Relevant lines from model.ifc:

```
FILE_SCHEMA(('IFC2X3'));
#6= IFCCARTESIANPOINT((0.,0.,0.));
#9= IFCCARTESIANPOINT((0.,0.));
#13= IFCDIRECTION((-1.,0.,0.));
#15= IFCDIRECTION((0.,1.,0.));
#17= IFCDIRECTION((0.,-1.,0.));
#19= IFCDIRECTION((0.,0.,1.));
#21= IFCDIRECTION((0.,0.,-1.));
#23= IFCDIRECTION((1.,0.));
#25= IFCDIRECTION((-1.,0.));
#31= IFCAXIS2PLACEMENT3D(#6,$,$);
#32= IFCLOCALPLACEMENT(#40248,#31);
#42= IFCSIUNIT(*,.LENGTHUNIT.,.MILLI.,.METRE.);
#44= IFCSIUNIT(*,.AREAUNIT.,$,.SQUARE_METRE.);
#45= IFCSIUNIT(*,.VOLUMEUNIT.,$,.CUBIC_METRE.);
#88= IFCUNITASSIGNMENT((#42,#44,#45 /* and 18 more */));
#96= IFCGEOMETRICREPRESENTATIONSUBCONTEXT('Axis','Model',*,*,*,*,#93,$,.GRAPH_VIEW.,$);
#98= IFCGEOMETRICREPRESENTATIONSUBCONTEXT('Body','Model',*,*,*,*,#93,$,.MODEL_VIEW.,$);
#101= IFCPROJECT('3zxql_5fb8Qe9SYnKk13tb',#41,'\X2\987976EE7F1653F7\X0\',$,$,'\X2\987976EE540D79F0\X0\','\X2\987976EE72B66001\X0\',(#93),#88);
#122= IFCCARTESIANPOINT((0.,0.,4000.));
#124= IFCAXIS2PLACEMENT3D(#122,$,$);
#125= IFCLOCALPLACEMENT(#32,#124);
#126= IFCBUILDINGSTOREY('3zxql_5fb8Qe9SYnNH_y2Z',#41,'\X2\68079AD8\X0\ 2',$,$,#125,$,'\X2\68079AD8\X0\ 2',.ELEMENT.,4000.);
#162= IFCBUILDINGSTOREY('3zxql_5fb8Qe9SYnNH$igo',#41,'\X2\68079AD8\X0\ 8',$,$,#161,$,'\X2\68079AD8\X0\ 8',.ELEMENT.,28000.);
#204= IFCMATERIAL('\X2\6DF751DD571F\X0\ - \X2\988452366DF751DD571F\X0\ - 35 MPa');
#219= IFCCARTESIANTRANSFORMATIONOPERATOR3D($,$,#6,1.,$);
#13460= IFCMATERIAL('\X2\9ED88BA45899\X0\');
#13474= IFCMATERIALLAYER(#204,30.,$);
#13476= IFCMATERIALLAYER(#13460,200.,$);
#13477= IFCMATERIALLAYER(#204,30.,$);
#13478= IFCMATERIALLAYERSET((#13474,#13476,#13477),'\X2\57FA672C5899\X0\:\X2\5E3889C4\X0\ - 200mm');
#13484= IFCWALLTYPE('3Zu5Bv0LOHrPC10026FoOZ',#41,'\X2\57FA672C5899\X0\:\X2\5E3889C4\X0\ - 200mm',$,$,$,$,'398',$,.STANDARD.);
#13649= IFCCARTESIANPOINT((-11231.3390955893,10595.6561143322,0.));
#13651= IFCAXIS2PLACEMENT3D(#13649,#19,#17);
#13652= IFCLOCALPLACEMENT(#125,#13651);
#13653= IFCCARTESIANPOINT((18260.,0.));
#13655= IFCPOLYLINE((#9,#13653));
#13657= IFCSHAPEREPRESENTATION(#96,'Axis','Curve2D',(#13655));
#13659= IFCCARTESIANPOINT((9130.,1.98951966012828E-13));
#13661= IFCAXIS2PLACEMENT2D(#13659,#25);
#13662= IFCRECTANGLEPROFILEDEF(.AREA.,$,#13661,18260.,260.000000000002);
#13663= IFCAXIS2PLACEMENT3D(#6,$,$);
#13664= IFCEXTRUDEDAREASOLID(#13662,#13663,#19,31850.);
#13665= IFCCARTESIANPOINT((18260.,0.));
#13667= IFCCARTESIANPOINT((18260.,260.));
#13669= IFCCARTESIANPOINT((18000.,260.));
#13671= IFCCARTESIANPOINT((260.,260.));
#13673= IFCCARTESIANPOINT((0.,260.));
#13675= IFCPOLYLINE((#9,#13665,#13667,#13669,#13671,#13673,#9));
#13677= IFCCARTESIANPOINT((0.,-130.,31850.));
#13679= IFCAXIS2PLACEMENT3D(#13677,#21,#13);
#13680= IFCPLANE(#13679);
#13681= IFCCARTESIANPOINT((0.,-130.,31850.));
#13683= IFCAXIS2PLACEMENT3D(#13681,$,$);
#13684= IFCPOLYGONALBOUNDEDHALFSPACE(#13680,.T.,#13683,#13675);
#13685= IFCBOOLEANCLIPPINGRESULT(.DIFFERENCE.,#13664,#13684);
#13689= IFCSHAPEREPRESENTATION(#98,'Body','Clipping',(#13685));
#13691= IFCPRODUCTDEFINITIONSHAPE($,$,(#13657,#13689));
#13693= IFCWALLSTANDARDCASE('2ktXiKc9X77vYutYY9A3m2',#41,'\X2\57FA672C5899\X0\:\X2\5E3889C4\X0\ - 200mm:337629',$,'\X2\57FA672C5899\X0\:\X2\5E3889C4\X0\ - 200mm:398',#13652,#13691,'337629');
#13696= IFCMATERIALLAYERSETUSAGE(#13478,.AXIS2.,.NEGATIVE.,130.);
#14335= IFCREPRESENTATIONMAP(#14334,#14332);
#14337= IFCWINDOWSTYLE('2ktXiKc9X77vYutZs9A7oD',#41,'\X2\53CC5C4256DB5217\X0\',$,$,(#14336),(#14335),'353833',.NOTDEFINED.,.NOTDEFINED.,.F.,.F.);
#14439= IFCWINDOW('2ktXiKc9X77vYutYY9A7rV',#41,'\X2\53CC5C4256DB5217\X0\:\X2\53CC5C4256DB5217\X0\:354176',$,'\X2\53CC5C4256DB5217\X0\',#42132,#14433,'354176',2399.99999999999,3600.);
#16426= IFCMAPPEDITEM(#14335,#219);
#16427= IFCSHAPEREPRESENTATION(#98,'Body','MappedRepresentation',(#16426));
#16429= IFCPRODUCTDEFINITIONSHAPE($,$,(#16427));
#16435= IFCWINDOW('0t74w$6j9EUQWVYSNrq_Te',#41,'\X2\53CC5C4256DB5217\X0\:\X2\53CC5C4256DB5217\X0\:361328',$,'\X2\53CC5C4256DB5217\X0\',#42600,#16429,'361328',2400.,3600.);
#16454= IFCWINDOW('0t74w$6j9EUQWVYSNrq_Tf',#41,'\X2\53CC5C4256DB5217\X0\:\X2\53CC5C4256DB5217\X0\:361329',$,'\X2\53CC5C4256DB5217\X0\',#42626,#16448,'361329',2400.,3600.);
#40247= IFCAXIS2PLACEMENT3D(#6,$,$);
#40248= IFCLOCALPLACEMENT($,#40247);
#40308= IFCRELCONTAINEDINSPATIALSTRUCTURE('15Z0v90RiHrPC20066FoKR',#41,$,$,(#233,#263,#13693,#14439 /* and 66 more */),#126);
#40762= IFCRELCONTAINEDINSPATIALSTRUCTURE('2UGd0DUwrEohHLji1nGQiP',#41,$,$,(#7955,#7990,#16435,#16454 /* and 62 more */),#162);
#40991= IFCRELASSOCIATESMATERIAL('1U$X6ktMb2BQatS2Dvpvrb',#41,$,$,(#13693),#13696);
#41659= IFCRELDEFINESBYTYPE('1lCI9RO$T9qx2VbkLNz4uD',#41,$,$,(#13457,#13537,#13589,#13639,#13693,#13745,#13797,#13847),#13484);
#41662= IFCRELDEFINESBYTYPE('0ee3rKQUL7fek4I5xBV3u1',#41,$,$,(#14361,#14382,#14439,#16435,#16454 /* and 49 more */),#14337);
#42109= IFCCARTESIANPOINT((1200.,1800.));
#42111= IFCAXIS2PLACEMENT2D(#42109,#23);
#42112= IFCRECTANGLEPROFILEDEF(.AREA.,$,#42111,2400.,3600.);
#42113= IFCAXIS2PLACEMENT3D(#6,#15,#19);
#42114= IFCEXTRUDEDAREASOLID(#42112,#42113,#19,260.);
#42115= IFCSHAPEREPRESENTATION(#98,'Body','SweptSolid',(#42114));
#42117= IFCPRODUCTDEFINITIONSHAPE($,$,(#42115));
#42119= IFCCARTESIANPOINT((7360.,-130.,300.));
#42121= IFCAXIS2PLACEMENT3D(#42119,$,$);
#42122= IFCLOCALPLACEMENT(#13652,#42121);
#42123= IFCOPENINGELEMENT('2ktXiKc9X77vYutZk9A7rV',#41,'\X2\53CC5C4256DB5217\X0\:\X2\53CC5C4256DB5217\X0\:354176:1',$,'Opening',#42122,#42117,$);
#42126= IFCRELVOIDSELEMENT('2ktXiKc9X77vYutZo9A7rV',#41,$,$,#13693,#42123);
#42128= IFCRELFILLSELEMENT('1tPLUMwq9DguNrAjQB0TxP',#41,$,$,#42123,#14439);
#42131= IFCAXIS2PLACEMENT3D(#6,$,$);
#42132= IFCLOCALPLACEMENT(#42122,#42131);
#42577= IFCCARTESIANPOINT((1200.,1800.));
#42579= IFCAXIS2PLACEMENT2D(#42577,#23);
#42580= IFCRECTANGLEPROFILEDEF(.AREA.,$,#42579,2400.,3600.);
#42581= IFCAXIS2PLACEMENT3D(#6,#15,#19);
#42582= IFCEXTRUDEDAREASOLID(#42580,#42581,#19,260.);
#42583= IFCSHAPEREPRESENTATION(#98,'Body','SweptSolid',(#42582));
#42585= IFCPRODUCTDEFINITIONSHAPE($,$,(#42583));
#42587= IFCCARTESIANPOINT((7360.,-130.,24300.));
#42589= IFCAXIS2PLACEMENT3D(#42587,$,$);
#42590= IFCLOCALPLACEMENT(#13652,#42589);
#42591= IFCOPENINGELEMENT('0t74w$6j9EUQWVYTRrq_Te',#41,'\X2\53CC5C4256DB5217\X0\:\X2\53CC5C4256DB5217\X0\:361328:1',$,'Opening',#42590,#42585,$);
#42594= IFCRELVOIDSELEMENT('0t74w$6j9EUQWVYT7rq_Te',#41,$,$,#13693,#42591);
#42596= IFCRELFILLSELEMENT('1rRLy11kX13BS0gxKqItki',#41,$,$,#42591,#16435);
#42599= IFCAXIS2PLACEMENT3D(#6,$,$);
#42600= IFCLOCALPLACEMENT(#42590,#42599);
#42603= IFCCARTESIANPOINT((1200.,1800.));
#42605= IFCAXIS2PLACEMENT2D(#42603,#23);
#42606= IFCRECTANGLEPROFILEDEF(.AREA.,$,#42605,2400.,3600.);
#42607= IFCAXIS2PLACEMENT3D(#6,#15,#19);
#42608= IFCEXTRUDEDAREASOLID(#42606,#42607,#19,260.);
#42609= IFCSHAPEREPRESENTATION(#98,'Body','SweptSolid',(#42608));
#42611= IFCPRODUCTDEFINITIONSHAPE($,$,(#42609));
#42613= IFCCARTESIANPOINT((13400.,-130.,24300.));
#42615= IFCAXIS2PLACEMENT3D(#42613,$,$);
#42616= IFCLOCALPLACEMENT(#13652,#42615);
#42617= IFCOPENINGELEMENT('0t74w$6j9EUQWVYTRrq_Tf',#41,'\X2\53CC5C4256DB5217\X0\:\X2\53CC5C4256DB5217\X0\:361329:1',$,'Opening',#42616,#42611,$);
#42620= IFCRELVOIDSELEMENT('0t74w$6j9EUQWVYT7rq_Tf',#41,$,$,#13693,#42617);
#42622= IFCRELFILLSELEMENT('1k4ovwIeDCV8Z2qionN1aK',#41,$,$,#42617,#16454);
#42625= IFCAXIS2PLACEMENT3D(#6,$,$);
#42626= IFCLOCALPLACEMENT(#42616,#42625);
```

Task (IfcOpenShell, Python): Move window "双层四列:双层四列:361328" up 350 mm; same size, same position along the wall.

```python
import numpy as np
import ifcopenshell
import ifcopenshell.api.geometry
import ifcopenshell.util.placement
import ifcopenshell.util.unit

model = ifcopenshell.open("model.ifc")
unit_scale = ifcopenshell.util.unit.calculate_unit_scale(model)

window = model.by_guid("0t74w$6j9EUQWVYSNrq_Te")
opening = window.FillsVoids[0].RelatingOpeningElement
dz = 350.0

shift = np.array([0.0, 0.0, dz])
# The window is placed relative to its opening, so it follows when the opening moves.
matrix = ifcopenshell.util.placement.get_local_placement(opening.ObjectPlacement)
matrix[:3, 3] += shift
ifcopenshell.api.geometry.edit_object_placement(
    model, product=opening, matrix=matrix, is_si=False, should_transform_children=True
)

print(f"moved by {dz * unit_scale:+.3f} m")

model.write("model_updated.ifc")
```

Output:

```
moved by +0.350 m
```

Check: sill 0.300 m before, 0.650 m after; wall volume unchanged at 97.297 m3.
